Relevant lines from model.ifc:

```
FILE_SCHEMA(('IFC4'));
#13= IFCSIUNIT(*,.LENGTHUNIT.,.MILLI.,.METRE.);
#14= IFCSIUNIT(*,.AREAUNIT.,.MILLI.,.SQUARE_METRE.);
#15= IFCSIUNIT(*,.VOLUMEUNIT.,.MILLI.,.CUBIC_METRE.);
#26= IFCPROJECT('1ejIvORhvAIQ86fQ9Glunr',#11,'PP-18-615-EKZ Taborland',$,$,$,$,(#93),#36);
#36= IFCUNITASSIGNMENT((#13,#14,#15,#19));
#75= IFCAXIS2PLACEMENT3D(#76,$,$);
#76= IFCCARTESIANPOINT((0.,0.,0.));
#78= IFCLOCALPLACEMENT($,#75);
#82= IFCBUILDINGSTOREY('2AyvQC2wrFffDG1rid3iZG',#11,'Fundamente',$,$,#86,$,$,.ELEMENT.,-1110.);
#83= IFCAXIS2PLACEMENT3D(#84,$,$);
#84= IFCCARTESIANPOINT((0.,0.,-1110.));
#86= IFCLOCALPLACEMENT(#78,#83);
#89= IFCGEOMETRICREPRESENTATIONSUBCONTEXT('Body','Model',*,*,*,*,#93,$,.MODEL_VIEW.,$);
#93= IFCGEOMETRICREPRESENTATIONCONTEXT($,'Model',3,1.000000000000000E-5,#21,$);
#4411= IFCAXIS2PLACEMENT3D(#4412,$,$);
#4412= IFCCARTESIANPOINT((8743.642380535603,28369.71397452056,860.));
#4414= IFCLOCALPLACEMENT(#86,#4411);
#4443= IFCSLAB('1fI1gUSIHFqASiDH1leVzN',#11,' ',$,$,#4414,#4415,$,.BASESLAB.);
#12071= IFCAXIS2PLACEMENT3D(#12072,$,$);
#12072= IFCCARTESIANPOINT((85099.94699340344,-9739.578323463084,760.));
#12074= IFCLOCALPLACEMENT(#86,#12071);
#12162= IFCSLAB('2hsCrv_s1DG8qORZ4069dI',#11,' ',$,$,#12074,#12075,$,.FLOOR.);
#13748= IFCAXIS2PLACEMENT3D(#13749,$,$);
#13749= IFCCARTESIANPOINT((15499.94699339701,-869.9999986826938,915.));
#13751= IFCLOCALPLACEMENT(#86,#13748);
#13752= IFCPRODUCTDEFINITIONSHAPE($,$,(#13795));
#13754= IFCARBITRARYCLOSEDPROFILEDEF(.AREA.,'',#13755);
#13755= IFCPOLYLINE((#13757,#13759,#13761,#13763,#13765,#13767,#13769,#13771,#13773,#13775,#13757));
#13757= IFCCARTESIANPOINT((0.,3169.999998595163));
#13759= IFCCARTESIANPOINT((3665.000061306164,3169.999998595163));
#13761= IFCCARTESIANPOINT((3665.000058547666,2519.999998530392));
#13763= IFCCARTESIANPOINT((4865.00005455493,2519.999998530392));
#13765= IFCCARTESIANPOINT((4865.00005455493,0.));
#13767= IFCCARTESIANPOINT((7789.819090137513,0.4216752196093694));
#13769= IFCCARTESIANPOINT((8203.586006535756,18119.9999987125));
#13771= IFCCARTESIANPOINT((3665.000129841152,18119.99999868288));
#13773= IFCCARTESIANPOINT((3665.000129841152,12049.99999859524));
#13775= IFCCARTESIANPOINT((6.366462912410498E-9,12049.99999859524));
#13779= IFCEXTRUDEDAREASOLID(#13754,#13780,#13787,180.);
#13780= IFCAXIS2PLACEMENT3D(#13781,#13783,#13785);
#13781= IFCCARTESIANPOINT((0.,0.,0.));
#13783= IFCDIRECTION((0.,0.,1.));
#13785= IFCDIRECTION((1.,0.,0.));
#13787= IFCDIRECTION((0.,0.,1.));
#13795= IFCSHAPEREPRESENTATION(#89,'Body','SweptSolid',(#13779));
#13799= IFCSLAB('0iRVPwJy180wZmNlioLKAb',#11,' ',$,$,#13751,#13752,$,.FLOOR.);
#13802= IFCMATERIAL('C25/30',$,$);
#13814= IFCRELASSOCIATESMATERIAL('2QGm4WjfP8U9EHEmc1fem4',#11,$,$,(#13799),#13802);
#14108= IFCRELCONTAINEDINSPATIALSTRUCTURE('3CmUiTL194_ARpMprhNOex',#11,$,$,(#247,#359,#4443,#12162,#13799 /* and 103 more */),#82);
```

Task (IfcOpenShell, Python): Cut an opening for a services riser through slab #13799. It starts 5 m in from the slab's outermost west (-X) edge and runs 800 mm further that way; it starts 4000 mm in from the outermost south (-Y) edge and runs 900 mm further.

```python
import numpy as np
import ifcopenshell
import ifcopenshell.api.feature
import ifcopenshell.api.geometry
import ifcopenshell.api.root
import ifcopenshell.geom
import ifcopenshell.util.placement
import ifcopenshell.util.representation
import ifcopenshell.util.shape
import ifcopenshell.util.unit

model = ifcopenshell.open("model.ifc")
unit_scale = ifcopenshell.util.unit.calculate_unit_scale(model)
settings = ifcopenshell.geom.settings()


def volume(element):
    """Net volume in cubic metres, openings subtracted."""
    shape = ifcopenshell.geom.create_shape(settings, element)
    return ifcopenshell.util.shape.get_volume(shape.geometry)


slab = model.by_id(13799)
before = volume(slab)

# Extent in the slab's own axes, in metres. The edges named are its -X and -Y sides.
slab_shape = ifcopenshell.geom.create_shape(settings, slab)
vertices = ifcopenshell.util.shape.get_vertices(slab_shape.geometry)
x_min, y_min, bottom = vertices.min(axis=0)
top = vertices[:, 2].max()

opening = ifcopenshell.api.root.create_entity(model, ifc_class="IfcOpeningElement", name="Services riser opening", predefined_type="OPENING")
context = ifcopenshell.util.representation.get_context(model, "Model", "Body", "MODEL_VIEW")
width, depth = 0.8, 0.9
outline = [(0.0, 0.0), (width, 0.0), (width, depth), (0.0, depth), (0.0, 0.0)]
# Overshoot both faces by 50 mm so the cut is clean.
shape = ifcopenshell.api.geometry.add_slab_representation(
    model, context=context, depth=top - bottom + 0.1, polyline=outline
)
ifcopenshell.api.geometry.assign_representation(model, product=opening, representation=shape)

matrix = ifcopenshell.util.placement.get_local_placement(slab.ObjectPlacement)
matrix[:, 3] = matrix @ np.append(np.array([x_min + 5, y_min + 4, bottom - 0.05]) / unit_scale, 1.0)
ifcopenshell.api.geometry.edit_object_placement(model, product=opening, matrix=matrix, is_si=False)
ifcopenshell.api.feature.add_feature(model, feature=opening, element=slab)

after = volume(slab)

print(f"slab volume {before:.3f} -> {after:.3f} m3")

model.write("model-out.ifc")
```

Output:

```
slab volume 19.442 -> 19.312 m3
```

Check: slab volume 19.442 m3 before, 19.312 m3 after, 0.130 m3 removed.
